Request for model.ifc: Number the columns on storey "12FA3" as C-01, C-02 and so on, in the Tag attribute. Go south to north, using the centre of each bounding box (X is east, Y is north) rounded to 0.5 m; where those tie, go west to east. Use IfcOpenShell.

First a look at what the model holds.

```python
import ifcopenshell
import ifcopenshell.util.element
import ifcopenshell.util.placement

model = ifcopenshell.open("model.ifc")
print(model.schema)
storey = next(s for s in model.by_type("IfcBuildingStorey") if s.Name == "12FA3")
columns = [e for e in ifcopenshell.util.element.get_decomposition(storey) if e.is_a("IfcColumn")]
for e in sorted(columns, key=lambda e: e.id()):
    origin = ifcopenshell.util.placement.get_local_placement(e.ObjectPlacement)[:3, 3]
    print(e.id(), e.Tag, e.Name, origin.round(2) + 0.0, sep=" | ")
```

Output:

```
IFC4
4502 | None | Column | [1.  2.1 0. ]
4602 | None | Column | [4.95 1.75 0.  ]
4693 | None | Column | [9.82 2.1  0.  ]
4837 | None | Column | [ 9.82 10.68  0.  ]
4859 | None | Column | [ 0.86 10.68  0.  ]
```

```python
import ifcopenshell
import ifcopenshell.geom
import ifcopenshell.util.element
import ifcopenshell.util.shape

model = ifcopenshell.open("model.ifc")
settings = ifcopenshell.geom.settings()
settings.set("use-world-coords", True)


def centre(element):
    shape = ifcopenshell.geom.create_shape(settings, element)
    return ifcopenshell.util.shape.get_bbox_centroid(shape.geometry)


storey = next(s for s in model.by_type("IfcBuildingStorey") if s.Name == "12FA3")
columns = [e for e in ifcopenshell.util.element.get_decomposition(storey) if e.is_a("IfcColumn")]

# Insertion points can sit at a corner or the storey origin, so sort by the geometry (in metres).
centres = {e: centre(e) for e in columns}
columns.sort(key=lambda e: (round(centres[e][1] / 0.5), centres[e][0]))

for i, e in enumerate(columns, start=1):
    number = f"C-{i:02d}"
    e.Tag = number
    print(e.id(), number)

model.write("model_edited.ifc")
```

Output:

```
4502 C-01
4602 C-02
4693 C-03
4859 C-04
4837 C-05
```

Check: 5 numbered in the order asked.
